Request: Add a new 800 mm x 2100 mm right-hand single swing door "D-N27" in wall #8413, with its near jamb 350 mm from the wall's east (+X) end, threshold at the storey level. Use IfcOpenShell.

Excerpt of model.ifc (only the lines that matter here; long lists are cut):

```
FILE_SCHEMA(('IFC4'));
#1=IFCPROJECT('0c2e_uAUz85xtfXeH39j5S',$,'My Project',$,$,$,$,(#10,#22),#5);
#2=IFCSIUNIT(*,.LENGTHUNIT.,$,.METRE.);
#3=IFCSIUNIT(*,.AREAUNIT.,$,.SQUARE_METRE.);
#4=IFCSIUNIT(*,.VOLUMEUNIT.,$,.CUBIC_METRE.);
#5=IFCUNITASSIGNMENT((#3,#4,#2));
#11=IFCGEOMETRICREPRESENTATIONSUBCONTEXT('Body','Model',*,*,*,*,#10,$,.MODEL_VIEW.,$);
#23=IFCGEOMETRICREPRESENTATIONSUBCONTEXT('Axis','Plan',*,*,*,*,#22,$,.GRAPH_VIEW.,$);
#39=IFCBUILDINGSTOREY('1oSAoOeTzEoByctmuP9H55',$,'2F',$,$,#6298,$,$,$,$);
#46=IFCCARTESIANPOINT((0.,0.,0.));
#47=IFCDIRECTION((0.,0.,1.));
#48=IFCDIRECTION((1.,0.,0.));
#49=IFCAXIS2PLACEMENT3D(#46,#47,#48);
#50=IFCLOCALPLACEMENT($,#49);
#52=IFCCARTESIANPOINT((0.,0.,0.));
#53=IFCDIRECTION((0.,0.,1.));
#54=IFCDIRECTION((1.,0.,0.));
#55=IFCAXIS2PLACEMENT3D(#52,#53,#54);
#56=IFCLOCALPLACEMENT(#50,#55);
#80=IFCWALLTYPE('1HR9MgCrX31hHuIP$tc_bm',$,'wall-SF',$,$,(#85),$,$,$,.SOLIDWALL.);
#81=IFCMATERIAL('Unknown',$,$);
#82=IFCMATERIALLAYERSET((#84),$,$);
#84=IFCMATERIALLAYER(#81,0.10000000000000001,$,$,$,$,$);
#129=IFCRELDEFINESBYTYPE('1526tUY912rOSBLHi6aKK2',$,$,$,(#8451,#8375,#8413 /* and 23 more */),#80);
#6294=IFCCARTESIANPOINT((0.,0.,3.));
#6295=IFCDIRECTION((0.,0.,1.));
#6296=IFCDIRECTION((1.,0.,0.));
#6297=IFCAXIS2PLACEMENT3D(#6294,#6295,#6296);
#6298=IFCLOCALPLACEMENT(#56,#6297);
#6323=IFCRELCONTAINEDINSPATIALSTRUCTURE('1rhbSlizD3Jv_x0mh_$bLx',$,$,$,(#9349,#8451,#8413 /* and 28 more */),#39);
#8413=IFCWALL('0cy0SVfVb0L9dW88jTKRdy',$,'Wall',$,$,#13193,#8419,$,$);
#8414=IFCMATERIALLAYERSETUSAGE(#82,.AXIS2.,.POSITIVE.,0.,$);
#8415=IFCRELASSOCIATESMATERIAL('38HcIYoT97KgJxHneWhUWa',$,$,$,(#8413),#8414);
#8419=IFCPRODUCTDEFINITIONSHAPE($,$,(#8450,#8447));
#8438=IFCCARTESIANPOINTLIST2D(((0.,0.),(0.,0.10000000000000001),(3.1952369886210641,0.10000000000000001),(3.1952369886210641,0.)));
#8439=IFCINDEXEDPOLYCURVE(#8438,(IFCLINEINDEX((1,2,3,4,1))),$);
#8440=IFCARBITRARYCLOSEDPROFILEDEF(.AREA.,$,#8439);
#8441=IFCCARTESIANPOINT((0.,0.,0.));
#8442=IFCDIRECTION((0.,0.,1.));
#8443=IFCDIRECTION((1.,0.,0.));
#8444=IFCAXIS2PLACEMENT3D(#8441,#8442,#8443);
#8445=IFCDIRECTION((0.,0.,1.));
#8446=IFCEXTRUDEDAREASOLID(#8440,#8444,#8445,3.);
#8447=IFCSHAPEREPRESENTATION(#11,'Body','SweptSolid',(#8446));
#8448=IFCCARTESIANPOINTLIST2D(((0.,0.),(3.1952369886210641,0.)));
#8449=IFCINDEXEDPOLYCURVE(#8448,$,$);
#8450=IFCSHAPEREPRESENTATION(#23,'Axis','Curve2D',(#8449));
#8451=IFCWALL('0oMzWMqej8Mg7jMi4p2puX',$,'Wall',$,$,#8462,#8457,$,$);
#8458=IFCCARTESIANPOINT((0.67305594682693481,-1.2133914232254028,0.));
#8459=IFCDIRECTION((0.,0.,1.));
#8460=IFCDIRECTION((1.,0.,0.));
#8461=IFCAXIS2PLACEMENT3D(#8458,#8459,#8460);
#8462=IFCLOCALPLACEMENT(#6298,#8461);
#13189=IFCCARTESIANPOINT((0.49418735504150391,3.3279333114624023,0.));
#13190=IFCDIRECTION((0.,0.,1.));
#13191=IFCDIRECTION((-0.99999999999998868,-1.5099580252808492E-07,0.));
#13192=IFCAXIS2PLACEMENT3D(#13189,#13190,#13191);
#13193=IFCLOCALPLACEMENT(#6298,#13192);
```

```python
import numpy as np
import ifcopenshell
import ifcopenshell.api.feature
import ifcopenshell.api.geometry
import ifcopenshell.api.root
import ifcopenshell.api.spatial
import ifcopenshell.geom
import ifcopenshell.util.element
import ifcopenshell.util.placement
import ifcopenshell.util.representation
import ifcopenshell.util.shape
import ifcopenshell.util.unit

model = ifcopenshell.open("model.ifc")
unit_scale = ifcopenshell.util.unit.calculate_unit_scale(model)
settings = ifcopenshell.geom.settings()


def volume(element):
    """Net volume in cubic metres, openings subtracted."""
    shape = ifcopenshell.geom.create_shape(settings, element)
    return ifcopenshell.util.shape.get_volume(shape.geometry)


wall = model.by_guid("0cy0SVfVb0L9dW88jTKRdy")
storey = ifcopenshell.util.element.get_container(wall, ifc_class="IfcBuildingStorey")
context = ifcopenshell.util.representation.get_context(model, "Model", "Body", "MODEL_VIEW")
before = volume(wall)

width, height, from_end, sill = 0.8, 2.1, 0.35, 0.0  # metres

# The wall runs along its own X axis, and the end named is its -X end.
wall_shape = ifcopenshell.geom.create_shape(settings, wall)
x, y, z = ifcopenshell.util.shape.get_vertices(wall_shape.geometry).T
start = x.min() + from_end
face, thickness = float(y.min()), float(y.max() - y.min())
wall_matrix = ifcopenshell.util.placement.get_local_placement(wall.ObjectPlacement)
level = ifcopenshell.util.placement.get_local_placement(storey.ObjectPlacement)[2, 3]


def in_wall(x, y):
    """Placement at x, y metres in the wall's axes, at sill height."""
    matrix = wall_matrix.copy()
    matrix[:, 3] = wall_matrix @ np.array([x / unit_scale, y / unit_scale, 0.0, 1.0])
    matrix[2, 3] = level + sill / unit_scale
    return matrix


# Opening: a box that overshoots both wall faces by 50 mm.
opening = ifcopenshell.api.root.create_entity(model, ifc_class="IfcOpeningElement", predefined_type="OPENING")
box = ifcopenshell.api.geometry.add_wall_representation(
    model, context=context, length=width, height=height, thickness=thickness + 0.1
)
ifcopenshell.api.geometry.assign_representation(model, product=opening, representation=box)
ifcopenshell.api.geometry.edit_object_placement(model, product=opening, matrix=in_wall(start, face - 0.05), is_si=False)
ifcopenshell.api.feature.add_feature(model, feature=opening, element=wall)

door = ifcopenshell.api.root.create_entity(model, ifc_class="IfcDoor", name="D-N27", predefined_type="DOOR")
door.OverallWidth, door.OverallHeight = width / unit_scale, height / unit_scale
door.OperationType = "SINGLE_SWING_RIGHT"
body = ifcopenshell.api.geometry.add_door_representation(
    model,
    context=context,
    overall_width=door.OverallWidth,
    overall_height=door.OverallHeight,
    operation_type="SINGLE_SWING_RIGHT",
    lining_properties={"LiningDepth": thickness / unit_scale, "ThresholdDepth": thickness / unit_scale},
)
ifcopenshell.api.geometry.assign_representation(model, product=door, representation=body)
ifcopenshell.api.spatial.assign_container(model, products=[door], relating_structure=storey)
ifcopenshell.api.feature.add_filling(model, opening=opening, element=door)

# The lining spans the wall, so the door starts at the wall face.
ifcopenshell.api.geometry.edit_object_placement(model, product=door, matrix=in_wall(start, face), is_si=False)

after = volume(wall)

print(f"wall volume {before:.3f} -> {after:.3f} m3")

model.write("model_rev.ifc")
```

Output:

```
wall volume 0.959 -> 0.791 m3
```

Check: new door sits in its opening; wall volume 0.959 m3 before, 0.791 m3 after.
